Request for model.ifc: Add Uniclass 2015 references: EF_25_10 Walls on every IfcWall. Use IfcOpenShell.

First a look at what the model holds.

```python
import ifcopenshell

model = ifcopenshell.open("model.ifc")
print(model.schema)
print("classifications:", [c.Name for c in model.by_type("IfcClassification")])
for ifc_class in ("IfcDoor", "IfcRoof", "IfcStair", "IfcWall", "IfcWindow"):
    print(ifc_class, len(model.by_type(ifc_class)))
```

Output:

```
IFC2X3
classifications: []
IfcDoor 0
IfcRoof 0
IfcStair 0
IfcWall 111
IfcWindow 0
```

```python
import ifcopenshell
import ifcopenshell.api.classification

model = ifcopenshell.open("model.ifc")

# IFC2X3 requires Source and Edition and has no link from the project to the system.
system = model.create_entity("IfcClassification", Source="NBS", Edition="2015", Name="Uniclass 2015")

codes = {
    "IfcWall": ("EF_25_10", "Walls"),
}
for ifc_class, (code, name) in codes.items():
    products = model.by_type(ifc_class)
    ifcopenshell.api.classification.add_reference(
        model, products=products, classification=system, identification=code, name=name
    )
    print(code, len(products))

model.write("model_v2.ifc")
```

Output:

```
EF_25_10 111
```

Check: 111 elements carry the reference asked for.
